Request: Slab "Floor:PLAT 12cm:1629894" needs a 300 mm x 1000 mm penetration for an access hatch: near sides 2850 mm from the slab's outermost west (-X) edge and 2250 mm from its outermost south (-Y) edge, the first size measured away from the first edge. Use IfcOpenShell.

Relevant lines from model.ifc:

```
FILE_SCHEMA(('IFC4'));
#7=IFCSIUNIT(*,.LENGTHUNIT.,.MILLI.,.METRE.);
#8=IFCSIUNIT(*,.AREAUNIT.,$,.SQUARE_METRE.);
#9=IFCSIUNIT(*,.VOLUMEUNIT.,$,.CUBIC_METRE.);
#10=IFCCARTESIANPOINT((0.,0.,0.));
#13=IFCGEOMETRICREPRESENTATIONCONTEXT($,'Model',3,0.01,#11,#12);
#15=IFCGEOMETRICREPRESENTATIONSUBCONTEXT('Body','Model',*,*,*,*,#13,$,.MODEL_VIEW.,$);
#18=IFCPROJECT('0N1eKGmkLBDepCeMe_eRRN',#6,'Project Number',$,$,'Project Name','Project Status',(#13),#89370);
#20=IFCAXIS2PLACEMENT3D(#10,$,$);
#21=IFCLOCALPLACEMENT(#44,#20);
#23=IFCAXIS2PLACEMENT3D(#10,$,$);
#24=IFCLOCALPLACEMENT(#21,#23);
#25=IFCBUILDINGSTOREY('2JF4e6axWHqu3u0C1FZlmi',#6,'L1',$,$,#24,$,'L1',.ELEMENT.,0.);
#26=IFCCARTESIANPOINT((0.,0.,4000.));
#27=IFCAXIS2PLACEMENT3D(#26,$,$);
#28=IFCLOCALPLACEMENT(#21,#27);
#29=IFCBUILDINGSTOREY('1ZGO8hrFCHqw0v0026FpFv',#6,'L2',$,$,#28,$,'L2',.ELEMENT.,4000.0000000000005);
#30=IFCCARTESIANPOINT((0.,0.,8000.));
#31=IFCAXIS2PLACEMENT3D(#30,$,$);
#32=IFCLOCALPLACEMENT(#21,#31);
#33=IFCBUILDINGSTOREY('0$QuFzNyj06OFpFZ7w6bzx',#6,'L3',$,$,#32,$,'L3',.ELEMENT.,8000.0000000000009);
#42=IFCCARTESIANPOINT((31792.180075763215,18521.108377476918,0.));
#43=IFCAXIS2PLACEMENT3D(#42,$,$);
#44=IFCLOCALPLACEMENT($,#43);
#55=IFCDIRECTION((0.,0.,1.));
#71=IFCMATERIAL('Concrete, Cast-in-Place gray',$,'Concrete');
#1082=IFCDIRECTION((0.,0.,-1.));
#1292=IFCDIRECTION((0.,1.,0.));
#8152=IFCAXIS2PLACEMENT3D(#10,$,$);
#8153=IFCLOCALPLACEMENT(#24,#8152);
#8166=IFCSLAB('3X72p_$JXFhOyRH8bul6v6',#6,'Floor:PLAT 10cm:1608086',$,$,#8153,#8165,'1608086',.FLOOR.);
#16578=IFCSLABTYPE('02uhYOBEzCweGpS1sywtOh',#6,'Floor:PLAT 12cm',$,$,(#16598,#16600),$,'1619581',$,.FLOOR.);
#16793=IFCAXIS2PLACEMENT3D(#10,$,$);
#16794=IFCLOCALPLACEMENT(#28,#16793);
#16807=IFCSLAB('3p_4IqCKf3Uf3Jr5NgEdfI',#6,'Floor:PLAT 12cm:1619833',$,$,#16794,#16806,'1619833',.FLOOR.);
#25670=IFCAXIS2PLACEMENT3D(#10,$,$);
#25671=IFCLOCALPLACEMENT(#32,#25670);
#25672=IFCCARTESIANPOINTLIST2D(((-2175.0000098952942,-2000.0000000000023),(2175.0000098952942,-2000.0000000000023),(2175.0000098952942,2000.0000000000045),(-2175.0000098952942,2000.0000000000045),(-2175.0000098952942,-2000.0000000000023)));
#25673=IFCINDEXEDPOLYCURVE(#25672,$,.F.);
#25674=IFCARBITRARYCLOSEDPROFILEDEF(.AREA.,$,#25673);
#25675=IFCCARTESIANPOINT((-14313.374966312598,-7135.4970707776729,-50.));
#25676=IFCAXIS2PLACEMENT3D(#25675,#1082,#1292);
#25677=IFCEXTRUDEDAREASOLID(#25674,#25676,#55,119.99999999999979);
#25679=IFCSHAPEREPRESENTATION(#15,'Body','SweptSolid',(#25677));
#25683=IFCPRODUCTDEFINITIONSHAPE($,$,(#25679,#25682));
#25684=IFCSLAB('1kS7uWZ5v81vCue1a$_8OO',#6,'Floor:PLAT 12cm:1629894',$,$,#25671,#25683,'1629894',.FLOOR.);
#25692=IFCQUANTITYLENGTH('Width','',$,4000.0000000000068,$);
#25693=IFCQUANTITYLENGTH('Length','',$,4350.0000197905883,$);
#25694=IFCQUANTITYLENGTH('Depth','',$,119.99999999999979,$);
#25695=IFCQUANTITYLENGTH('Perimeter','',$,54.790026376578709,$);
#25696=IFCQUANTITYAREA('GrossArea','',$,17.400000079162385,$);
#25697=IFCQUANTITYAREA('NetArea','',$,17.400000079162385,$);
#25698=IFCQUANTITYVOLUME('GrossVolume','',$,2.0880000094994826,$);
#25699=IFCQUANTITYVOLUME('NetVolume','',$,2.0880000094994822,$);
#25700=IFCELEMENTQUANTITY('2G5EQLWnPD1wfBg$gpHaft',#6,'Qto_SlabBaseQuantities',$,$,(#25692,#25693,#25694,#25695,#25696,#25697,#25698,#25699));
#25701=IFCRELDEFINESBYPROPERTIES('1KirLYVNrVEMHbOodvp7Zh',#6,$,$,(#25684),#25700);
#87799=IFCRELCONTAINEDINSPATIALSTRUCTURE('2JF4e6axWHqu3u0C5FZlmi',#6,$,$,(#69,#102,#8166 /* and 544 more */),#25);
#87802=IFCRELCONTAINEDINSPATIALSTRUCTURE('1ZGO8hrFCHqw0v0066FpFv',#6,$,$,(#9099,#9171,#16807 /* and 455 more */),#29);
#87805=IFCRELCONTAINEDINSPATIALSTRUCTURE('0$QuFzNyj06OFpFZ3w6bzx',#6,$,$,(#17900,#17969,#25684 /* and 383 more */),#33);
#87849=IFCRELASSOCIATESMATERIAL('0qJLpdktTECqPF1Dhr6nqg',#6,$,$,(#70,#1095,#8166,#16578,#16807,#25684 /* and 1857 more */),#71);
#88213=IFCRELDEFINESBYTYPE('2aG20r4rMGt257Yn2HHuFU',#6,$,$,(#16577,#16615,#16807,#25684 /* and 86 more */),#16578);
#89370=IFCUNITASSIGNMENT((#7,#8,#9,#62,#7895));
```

```python
import numpy as np
import ifcopenshell
import ifcopenshell.api.feature
import ifcopenshell.api.geometry
import ifcopenshell.api.pset
import ifcopenshell.api.root
import ifcopenshell.geom
import ifcopenshell.util.element
import ifcopenshell.util.placement
import ifcopenshell.util.representation
import ifcopenshell.util.shape
import ifcopenshell.util.unit

model = ifcopenshell.open("model.ifc")
unit_scale = ifcopenshell.util.unit.calculate_unit_scale(model)
area_scale = ifcopenshell.util.unit.calculate_unit_scale(model, "AREAUNIT")
volume_scale = ifcopenshell.util.unit.calculate_unit_scale(model, "VOLUMEUNIT")
settings = ifcopenshell.geom.settings()


def volume(element):
    """Net volume in cubic metres, openings subtracted."""
    shape = ifcopenshell.geom.create_shape(settings, element)
    return ifcopenshell.util.shape.get_volume(shape.geometry)


slab = model.by_guid("1kS7uWZ5v81vCue1a$_8OO")
before = volume(slab)

# Extent in the slab's own axes, in metres. The edges named are its -X and -Y sides.
slab_shape = ifcopenshell.geom.create_shape(settings, slab)
vertices = ifcopenshell.util.shape.get_vertices(slab_shape.geometry)
x_min, y_min, bottom = vertices.min(axis=0)
top = vertices[:, 2].max()

opening = ifcopenshell.api.root.create_entity(model, ifc_class="IfcOpeningElement", name="Access hatch opening", predefined_type="OPENING")
context = ifcopenshell.util.representation.get_context(model, "Model", "Body", "MODEL_VIEW")
width, depth = 0.3, 1
outline = [(0.0, 0.0), (width, 0.0), (width, depth), (0.0, depth), (0.0, 0.0)]
# Overshoot both faces by 50 mm so the cut is clean.
shape = ifcopenshell.api.geometry.add_slab_representation(
    model, context=context, depth=top - bottom + 0.1, polyline=outline
)
ifcopenshell.api.geometry.assign_representation(model, product=opening, representation=shape)

matrix = ifcopenshell.util.placement.get_local_placement(slab.ObjectPlacement)
matrix[:, 3] = matrix @ np.append(np.array([x_min + 2.85, y_min + 2.25, bottom - 0.05]) / unit_scale, 1.0)
ifcopenshell.api.geometry.edit_object_placement(model, product=opening, matrix=matrix, is_si=False)
ifcopenshell.api.feature.add_feature(model, feature=opening, element=slab)

after = volume(slab)

# Update the slab's stored quantities.
qto = model.by_id(ifcopenshell.util.element.get_pset(slab, "Qto_SlabBaseQuantities", should_inherit=False)["id"])
ifcopenshell.api.pset.edit_qto(model, qto=qto, properties={
    "NetArea": after / (top - bottom) / area_scale,
    "NetVolume": after / volume_scale,
})

print(f"slab volume {before:.3f} -> {after:.3f} m3")

model.write("model_v2.ifc")
```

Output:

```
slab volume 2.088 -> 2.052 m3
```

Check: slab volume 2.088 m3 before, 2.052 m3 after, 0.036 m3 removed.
